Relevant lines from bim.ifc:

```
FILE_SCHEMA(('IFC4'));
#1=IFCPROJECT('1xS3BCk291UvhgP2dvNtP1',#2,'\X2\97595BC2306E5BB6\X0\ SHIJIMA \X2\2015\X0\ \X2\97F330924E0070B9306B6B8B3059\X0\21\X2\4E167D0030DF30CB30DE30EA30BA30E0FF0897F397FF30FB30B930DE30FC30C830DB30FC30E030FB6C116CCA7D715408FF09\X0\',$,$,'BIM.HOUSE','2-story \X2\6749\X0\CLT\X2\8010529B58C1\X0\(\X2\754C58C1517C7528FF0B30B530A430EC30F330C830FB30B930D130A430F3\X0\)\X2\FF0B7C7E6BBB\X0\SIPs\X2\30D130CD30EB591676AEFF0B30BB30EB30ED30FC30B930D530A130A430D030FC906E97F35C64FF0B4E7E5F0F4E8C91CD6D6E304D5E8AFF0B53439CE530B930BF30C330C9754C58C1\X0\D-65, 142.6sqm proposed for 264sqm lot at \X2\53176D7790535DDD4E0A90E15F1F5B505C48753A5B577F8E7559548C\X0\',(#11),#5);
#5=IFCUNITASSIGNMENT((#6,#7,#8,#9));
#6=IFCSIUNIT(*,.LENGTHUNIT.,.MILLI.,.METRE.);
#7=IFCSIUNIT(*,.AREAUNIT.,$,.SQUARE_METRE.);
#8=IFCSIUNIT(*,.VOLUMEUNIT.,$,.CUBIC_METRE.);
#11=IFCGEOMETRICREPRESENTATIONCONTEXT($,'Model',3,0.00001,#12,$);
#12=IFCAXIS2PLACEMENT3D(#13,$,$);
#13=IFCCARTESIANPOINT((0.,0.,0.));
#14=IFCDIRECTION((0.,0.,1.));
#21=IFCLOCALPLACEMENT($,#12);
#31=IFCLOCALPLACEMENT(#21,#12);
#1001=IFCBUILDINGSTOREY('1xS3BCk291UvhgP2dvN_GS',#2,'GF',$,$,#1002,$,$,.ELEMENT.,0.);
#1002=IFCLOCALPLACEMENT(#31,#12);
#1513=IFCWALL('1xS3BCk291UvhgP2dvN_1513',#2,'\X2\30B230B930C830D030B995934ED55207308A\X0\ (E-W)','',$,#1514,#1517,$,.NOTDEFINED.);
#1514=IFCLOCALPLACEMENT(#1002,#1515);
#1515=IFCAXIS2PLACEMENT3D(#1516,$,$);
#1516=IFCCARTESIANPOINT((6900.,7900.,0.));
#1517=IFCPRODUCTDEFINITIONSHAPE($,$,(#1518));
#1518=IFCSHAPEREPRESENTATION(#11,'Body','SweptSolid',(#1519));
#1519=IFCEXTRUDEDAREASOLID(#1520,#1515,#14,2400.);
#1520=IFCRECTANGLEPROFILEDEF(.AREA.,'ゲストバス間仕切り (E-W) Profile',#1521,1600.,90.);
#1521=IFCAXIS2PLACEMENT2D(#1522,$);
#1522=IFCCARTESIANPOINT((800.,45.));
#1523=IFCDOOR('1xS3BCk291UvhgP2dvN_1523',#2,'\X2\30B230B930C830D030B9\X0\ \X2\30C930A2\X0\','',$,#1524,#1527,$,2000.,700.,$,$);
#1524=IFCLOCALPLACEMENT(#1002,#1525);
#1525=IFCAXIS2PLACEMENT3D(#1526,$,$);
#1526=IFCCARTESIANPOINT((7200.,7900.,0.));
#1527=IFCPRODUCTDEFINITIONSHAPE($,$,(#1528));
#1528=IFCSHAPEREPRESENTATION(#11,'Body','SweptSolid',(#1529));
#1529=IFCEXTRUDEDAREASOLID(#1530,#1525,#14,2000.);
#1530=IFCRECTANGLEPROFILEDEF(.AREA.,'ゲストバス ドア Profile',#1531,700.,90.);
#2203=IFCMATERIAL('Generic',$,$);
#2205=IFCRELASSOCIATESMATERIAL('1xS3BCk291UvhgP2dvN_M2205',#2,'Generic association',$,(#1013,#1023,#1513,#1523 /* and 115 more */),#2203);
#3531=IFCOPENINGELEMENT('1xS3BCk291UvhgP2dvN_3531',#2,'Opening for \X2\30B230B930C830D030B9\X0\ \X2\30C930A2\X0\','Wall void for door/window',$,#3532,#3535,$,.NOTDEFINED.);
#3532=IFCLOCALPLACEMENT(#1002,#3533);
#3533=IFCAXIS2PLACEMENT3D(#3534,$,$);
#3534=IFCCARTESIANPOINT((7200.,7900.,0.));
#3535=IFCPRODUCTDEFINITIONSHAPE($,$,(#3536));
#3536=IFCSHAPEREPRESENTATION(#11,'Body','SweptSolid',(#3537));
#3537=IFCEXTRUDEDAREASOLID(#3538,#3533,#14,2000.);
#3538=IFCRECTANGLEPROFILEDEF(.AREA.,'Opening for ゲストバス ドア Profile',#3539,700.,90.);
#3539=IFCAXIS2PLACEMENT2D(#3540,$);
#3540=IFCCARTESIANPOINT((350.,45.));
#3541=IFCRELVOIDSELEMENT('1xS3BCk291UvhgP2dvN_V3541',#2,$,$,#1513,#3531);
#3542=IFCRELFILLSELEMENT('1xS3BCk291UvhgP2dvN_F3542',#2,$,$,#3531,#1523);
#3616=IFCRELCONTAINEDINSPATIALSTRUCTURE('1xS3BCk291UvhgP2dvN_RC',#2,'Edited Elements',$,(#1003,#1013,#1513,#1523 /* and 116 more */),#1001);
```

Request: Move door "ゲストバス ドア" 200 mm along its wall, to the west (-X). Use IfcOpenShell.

```python
import ifcopenshell
import ifcopenshell.api.geometry
import ifcopenshell.util.placement
import ifcopenshell.util.unit

model = ifcopenshell.open("bim.ifc")
unit_scale = ifcopenshell.util.unit.calculate_unit_scale(model)

door = model.by_guid("1xS3BCk291UvhgP2dvN_1523")
opening = door.FillsVoids[0].RelatingOpeningElement
wall = opening.VoidsElements[0].RelatingBuildingElement

wall_matrix = ifcopenshell.util.placement.get_local_placement(wall.ObjectPlacement)
shift = wall_matrix[:3, 0] * -0.2 / unit_scale
before = ifcopenshell.util.placement.get_local_placement(door.ObjectPlacement)[:3, 3].copy()

# The door is not placed relative to its opening, so move both.
for product in (opening, door):
    matrix = ifcopenshell.util.placement.get_local_placement(product.ObjectPlacement)
    matrix[:3, 3] += shift
    ifcopenshell.api.geometry.edit_object_placement(model, product=product, matrix=matrix, is_si=False)

after = ifcopenshell.util.placement.get_local_placement(door.ObjectPlacement)[:3, 3]
print("door moved by", (after - before).round(3) + 0.0)

model.write("bim_edited.ifc")
```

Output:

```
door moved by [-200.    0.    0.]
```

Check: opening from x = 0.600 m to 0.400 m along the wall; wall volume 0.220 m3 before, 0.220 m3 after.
